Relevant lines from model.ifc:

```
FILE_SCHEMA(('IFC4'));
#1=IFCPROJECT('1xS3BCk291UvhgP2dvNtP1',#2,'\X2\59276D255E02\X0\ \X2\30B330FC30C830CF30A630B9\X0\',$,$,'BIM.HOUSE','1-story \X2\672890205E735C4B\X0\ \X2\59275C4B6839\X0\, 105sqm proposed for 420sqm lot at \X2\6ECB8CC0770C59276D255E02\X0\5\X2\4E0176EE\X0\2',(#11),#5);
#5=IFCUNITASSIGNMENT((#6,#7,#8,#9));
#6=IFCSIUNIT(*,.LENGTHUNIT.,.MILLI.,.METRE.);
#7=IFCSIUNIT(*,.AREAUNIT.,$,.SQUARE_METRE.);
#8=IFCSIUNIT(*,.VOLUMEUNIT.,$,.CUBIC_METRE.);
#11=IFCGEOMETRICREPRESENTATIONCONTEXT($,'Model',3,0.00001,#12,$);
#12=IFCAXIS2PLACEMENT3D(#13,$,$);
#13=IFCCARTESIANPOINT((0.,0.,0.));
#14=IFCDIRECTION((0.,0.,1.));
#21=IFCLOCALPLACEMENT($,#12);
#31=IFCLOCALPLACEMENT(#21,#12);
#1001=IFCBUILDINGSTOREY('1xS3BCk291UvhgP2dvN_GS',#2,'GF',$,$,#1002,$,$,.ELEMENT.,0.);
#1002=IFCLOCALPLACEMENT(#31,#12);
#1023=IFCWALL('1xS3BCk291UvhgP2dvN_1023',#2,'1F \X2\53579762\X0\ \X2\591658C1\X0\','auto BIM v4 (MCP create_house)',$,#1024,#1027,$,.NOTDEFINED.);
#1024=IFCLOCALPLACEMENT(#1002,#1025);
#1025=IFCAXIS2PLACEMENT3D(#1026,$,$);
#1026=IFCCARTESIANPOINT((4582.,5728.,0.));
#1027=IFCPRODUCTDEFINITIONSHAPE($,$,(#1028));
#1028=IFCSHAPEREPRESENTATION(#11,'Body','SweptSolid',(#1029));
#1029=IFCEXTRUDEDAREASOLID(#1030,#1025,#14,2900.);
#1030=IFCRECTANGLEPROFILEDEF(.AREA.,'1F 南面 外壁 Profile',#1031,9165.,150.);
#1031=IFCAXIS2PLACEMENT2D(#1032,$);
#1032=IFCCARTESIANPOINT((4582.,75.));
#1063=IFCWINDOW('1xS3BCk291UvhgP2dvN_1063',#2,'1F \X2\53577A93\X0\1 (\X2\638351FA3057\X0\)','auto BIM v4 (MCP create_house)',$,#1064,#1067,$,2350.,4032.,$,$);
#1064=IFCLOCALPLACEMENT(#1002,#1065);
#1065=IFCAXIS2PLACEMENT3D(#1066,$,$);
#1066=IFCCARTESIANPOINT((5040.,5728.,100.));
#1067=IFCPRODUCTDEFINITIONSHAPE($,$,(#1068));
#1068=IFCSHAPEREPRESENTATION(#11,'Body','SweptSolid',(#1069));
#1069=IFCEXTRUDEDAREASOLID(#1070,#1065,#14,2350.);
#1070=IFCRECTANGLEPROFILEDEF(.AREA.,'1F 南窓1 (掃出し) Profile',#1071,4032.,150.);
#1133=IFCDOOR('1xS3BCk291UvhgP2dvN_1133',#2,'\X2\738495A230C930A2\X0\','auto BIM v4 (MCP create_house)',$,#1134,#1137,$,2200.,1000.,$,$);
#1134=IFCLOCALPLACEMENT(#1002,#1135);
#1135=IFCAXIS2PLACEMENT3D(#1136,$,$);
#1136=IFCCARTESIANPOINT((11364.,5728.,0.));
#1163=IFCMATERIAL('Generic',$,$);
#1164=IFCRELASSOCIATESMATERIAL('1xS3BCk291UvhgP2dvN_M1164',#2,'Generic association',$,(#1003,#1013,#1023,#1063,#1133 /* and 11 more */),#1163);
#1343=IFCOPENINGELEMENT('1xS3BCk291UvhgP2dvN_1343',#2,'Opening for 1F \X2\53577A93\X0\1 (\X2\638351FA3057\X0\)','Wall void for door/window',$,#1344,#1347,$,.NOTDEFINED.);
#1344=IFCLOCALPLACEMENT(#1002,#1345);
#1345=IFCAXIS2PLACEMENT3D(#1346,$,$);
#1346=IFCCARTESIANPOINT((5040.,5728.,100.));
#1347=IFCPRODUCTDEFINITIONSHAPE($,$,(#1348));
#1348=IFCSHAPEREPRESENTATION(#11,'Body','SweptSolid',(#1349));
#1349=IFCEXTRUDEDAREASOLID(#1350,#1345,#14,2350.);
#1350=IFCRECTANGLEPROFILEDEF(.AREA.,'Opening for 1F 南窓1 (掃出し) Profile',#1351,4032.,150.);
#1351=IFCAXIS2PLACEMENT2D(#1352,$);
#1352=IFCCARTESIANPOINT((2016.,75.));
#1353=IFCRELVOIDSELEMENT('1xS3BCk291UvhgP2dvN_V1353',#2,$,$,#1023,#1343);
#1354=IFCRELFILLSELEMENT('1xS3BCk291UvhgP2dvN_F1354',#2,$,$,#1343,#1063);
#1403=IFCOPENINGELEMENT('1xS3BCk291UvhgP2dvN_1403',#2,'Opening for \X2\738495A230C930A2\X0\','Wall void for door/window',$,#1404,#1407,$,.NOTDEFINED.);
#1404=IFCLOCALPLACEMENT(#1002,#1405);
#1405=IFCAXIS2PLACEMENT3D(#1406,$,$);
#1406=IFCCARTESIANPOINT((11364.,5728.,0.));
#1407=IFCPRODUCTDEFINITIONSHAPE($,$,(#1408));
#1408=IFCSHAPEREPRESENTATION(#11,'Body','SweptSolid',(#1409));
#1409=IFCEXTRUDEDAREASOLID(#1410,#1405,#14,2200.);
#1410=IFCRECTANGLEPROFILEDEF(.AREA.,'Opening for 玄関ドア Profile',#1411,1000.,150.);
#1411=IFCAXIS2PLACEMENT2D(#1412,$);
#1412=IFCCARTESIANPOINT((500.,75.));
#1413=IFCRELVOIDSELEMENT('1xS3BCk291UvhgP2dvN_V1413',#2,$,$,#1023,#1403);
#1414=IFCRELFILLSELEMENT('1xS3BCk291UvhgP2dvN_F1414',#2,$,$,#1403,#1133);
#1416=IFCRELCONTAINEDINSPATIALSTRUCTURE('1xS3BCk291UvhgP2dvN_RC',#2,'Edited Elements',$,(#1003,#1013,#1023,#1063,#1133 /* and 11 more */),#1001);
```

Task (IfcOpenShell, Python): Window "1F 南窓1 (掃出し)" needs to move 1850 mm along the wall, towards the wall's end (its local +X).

```python
import ifcopenshell
import ifcopenshell.api.geometry
import ifcopenshell.util.placement
import ifcopenshell.util.unit

model = ifcopenshell.open("model.ifc")
unit_scale = ifcopenshell.util.unit.calculate_unit_scale(model)

window = model.by_id(1063)
opening = window.FillsVoids[0].RelatingOpeningElement
wall = opening.VoidsElements[0].RelatingBuildingElement

wall_matrix = ifcopenshell.util.placement.get_local_placement(wall.ObjectPlacement)
shift = wall_matrix[:3, 0] * 1.85 / unit_scale
before = ifcopenshell.util.placement.get_local_placement(window.ObjectPlacement)[:3, 3].copy()

# The window is not placed relative to its opening, so move both.
for product in (opening, window):
    matrix = ifcopenshell.util.placement.get_local_placement(product.ObjectPlacement)
    matrix[:3, 3] += shift
    ifcopenshell.api.geometry.edit_object_placement(model, product=product, matrix=matrix, is_si=False)

after = ifcopenshell.util.placement.get_local_placement(window.ObjectPlacement)[:3, 3]
print("window moved by", (after - before).round(3) + 0.0)

model.write("model-out.ifc")
```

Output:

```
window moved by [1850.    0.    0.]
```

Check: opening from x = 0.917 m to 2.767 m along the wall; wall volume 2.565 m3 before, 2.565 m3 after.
